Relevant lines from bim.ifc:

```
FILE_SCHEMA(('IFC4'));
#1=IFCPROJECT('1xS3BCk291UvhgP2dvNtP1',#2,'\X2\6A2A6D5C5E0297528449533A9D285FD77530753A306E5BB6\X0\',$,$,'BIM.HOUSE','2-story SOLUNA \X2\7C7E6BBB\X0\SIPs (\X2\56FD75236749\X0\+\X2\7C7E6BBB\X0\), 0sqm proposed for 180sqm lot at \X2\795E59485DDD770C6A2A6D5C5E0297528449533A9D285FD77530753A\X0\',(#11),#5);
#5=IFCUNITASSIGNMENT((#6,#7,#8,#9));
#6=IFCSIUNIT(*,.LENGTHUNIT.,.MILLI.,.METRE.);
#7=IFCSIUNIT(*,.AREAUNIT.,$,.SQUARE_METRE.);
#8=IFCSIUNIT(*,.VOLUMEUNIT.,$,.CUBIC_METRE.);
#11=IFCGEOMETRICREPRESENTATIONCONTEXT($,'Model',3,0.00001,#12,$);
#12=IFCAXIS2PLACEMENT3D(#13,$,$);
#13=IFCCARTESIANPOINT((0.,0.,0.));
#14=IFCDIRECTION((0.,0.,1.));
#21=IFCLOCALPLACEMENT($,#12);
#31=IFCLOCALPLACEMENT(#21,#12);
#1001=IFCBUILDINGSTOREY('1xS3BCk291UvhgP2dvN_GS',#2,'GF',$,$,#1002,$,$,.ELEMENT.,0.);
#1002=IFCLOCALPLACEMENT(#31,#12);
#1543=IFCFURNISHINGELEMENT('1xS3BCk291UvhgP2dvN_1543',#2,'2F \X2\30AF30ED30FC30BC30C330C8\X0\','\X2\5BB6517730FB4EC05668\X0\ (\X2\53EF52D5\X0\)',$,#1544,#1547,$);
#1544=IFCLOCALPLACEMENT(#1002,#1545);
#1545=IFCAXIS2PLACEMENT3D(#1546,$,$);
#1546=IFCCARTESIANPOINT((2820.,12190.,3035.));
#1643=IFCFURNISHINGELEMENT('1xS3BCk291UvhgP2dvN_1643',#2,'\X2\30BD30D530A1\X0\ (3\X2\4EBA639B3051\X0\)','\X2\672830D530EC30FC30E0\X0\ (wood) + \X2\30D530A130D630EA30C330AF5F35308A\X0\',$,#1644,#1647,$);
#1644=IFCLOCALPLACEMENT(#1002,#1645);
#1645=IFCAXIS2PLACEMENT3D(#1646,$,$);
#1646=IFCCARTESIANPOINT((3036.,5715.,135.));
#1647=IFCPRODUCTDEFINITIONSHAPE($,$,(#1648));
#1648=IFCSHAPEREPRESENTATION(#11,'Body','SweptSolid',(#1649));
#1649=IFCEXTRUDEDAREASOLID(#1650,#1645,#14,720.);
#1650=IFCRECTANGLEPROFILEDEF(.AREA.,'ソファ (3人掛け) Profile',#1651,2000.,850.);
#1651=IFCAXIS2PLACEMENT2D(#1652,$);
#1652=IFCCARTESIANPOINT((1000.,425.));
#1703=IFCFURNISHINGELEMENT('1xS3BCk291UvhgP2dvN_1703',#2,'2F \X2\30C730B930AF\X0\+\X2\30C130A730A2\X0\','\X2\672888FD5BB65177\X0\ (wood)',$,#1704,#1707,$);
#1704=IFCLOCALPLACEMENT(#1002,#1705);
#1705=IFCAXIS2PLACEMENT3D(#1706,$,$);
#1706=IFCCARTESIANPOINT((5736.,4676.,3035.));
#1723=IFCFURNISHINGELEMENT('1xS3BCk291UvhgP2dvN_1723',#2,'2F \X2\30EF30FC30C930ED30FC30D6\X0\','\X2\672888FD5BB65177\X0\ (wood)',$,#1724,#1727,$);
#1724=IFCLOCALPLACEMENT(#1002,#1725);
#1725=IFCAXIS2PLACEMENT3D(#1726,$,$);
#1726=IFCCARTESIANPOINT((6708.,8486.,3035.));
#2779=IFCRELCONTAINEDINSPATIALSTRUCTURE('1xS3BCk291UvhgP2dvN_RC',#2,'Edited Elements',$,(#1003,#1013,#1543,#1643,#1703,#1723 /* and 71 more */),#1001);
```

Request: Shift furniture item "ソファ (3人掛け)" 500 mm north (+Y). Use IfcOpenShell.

```python
import ifcopenshell
import ifcopenshell.api.geometry
import ifcopenshell.util.placement

model = ifcopenshell.open("bim.ifc")

item = model.by_guid("1xS3BCk291UvhgP2dvN_1643")
matrix = ifcopenshell.util.placement.get_local_placement(item.ObjectPlacement)
matrix[1, 3] += 500.0
ifcopenshell.api.geometry.edit_object_placement(model, product=item, matrix=matrix, is_si=False)

print(ifcopenshell.util.placement.get_local_placement(item.ObjectPlacement).round(3) + 0.0)

model.write("bim-out.ifc")
```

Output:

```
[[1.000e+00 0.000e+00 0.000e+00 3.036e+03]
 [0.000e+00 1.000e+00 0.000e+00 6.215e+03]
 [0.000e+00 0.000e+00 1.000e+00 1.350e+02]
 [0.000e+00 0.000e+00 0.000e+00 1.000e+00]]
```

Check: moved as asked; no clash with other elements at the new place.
